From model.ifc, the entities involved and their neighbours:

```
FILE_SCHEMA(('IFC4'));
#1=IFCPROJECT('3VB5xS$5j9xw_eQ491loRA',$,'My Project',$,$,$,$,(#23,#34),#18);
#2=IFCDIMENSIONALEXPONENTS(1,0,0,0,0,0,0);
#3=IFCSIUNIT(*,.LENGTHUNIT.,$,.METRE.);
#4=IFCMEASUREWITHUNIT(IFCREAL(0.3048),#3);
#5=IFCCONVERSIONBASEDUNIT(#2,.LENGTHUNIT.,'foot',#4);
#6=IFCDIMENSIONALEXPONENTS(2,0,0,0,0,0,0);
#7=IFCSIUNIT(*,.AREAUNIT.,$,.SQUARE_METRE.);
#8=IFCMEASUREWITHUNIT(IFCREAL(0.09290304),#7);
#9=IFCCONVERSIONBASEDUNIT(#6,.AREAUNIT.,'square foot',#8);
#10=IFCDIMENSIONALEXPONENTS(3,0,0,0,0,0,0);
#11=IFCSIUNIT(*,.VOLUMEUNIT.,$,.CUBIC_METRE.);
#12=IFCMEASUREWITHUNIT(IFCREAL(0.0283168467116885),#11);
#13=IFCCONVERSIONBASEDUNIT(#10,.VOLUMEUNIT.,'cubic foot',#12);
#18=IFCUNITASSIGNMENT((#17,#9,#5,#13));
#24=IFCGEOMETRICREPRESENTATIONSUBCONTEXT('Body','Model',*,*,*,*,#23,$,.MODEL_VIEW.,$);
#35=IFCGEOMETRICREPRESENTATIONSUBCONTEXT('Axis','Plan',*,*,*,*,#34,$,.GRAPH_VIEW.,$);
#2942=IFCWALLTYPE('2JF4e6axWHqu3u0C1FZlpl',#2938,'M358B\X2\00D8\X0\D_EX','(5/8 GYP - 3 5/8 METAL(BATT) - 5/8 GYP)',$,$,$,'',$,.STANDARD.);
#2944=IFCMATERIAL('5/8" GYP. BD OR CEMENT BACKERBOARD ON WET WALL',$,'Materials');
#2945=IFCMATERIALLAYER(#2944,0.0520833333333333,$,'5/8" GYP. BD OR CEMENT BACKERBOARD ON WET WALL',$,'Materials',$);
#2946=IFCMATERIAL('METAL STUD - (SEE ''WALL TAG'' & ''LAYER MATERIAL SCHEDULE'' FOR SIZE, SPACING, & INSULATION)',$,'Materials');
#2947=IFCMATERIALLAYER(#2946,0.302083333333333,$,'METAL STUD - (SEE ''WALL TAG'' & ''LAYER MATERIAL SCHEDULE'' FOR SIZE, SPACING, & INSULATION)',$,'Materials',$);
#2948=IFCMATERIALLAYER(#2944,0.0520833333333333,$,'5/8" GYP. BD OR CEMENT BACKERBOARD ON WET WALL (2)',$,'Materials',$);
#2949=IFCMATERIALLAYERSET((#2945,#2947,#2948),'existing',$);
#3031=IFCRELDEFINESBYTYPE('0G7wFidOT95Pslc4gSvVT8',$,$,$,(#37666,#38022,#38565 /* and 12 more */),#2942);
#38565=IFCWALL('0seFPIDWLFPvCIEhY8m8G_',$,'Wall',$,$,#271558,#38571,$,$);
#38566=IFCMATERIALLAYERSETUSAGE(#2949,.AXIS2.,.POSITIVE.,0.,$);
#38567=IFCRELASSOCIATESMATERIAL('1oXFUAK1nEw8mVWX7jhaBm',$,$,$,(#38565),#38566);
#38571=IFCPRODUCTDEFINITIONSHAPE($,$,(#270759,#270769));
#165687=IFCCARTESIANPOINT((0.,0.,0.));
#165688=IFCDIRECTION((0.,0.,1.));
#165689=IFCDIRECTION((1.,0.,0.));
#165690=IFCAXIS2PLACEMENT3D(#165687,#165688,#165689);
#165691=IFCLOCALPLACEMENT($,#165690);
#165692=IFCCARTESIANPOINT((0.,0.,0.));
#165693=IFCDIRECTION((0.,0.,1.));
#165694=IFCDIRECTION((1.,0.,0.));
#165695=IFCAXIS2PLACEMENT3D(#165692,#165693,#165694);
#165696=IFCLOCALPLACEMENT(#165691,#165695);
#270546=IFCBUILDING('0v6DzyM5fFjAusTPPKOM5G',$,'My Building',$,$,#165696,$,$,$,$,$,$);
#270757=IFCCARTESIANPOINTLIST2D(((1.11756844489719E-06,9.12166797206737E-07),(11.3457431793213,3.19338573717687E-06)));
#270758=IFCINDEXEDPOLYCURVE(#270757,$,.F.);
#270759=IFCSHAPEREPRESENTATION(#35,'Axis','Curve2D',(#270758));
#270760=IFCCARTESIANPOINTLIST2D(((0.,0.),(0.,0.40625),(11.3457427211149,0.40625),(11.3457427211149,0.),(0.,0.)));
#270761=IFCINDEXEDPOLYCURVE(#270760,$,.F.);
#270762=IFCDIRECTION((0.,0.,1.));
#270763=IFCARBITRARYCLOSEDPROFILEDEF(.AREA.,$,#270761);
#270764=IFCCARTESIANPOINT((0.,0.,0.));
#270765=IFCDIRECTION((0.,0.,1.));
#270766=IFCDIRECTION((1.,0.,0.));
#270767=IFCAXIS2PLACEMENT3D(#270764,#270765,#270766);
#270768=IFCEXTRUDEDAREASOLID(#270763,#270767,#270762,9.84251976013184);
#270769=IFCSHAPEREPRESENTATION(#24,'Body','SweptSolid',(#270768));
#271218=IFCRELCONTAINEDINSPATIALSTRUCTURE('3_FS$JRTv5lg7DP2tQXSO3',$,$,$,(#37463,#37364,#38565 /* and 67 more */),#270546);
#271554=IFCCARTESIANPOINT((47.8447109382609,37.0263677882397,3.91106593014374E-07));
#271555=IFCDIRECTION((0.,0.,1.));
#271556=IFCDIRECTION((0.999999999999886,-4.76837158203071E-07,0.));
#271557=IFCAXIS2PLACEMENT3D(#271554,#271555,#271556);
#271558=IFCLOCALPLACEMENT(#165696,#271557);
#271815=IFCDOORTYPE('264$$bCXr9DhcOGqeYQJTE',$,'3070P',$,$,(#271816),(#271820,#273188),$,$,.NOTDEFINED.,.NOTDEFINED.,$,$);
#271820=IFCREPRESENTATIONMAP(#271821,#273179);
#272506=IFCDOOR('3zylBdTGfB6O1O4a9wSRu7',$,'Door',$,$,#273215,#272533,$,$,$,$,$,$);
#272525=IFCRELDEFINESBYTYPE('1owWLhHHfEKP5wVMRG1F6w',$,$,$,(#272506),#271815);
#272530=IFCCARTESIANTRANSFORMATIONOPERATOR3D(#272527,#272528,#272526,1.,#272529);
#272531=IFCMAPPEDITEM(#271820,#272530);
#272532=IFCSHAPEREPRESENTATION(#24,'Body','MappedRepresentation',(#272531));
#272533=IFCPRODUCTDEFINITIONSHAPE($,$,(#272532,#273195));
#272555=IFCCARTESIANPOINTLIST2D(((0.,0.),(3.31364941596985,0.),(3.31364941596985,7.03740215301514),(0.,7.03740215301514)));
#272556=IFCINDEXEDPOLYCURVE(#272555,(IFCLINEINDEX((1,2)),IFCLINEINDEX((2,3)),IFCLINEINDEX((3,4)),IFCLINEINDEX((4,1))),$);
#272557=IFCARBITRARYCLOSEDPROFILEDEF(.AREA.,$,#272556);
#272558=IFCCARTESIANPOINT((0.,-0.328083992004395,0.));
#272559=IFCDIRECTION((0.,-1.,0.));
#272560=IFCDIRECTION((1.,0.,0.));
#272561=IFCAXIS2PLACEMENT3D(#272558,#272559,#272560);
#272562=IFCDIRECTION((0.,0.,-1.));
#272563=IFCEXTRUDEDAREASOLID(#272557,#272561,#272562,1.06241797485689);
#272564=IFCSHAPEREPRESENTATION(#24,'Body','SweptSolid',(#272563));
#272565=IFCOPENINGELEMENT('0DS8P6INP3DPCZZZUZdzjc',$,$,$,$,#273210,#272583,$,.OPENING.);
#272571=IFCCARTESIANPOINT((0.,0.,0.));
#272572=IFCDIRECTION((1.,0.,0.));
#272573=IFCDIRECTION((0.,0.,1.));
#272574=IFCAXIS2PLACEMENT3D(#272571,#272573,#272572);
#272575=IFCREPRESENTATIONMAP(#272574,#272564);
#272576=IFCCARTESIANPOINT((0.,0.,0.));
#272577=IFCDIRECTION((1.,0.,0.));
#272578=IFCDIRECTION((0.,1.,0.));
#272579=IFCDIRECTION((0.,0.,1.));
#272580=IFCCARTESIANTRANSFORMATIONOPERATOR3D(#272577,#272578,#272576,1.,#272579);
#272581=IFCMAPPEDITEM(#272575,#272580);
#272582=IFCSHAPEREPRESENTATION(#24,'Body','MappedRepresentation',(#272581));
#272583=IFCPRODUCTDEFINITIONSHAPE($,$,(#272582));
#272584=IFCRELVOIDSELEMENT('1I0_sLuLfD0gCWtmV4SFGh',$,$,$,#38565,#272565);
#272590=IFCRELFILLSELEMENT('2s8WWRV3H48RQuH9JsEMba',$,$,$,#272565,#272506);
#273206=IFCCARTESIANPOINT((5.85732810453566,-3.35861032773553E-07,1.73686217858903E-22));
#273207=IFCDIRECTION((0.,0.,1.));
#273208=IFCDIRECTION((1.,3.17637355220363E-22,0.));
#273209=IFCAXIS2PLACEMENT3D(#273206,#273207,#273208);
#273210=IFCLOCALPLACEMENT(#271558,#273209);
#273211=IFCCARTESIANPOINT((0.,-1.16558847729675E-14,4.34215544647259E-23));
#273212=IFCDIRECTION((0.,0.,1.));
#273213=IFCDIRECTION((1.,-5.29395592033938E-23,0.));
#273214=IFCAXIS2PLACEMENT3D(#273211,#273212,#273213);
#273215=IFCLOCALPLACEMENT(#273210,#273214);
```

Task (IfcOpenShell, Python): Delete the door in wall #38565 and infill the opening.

```python
import ifcopenshell
import ifcopenshell.api.feature
import ifcopenshell.api.root
import ifcopenshell.geom
import ifcopenshell.util.shape

model = ifcopenshell.open("model.ifc")
settings = ifcopenshell.geom.settings()


def volume(element):
    """Net volume in cubic metres, openings subtracted."""
    shape = ifcopenshell.geom.create_shape(settings, element)
    return ifcopenshell.util.shape.get_volume(shape.geometry)


door = model.by_guid("3zylBdTGfB6O1O4a9wSRu7")
opening = door.FillsVoids[0].RelatingOpeningElement
wall = opening.VoidsElements[0].RelatingBuildingElement
before = volume(wall)

ifcopenshell.api.root.remove_product(model, product=door)
ifcopenshell.api.feature.remove_feature(model, feature=opening)

after = volume(wall)

print(f"wall volume {before:.3f} -> {after:.3f} m3")

model.write("model_rev.ifc")
```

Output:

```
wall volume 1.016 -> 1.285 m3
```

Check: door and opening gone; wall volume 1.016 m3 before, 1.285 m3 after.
